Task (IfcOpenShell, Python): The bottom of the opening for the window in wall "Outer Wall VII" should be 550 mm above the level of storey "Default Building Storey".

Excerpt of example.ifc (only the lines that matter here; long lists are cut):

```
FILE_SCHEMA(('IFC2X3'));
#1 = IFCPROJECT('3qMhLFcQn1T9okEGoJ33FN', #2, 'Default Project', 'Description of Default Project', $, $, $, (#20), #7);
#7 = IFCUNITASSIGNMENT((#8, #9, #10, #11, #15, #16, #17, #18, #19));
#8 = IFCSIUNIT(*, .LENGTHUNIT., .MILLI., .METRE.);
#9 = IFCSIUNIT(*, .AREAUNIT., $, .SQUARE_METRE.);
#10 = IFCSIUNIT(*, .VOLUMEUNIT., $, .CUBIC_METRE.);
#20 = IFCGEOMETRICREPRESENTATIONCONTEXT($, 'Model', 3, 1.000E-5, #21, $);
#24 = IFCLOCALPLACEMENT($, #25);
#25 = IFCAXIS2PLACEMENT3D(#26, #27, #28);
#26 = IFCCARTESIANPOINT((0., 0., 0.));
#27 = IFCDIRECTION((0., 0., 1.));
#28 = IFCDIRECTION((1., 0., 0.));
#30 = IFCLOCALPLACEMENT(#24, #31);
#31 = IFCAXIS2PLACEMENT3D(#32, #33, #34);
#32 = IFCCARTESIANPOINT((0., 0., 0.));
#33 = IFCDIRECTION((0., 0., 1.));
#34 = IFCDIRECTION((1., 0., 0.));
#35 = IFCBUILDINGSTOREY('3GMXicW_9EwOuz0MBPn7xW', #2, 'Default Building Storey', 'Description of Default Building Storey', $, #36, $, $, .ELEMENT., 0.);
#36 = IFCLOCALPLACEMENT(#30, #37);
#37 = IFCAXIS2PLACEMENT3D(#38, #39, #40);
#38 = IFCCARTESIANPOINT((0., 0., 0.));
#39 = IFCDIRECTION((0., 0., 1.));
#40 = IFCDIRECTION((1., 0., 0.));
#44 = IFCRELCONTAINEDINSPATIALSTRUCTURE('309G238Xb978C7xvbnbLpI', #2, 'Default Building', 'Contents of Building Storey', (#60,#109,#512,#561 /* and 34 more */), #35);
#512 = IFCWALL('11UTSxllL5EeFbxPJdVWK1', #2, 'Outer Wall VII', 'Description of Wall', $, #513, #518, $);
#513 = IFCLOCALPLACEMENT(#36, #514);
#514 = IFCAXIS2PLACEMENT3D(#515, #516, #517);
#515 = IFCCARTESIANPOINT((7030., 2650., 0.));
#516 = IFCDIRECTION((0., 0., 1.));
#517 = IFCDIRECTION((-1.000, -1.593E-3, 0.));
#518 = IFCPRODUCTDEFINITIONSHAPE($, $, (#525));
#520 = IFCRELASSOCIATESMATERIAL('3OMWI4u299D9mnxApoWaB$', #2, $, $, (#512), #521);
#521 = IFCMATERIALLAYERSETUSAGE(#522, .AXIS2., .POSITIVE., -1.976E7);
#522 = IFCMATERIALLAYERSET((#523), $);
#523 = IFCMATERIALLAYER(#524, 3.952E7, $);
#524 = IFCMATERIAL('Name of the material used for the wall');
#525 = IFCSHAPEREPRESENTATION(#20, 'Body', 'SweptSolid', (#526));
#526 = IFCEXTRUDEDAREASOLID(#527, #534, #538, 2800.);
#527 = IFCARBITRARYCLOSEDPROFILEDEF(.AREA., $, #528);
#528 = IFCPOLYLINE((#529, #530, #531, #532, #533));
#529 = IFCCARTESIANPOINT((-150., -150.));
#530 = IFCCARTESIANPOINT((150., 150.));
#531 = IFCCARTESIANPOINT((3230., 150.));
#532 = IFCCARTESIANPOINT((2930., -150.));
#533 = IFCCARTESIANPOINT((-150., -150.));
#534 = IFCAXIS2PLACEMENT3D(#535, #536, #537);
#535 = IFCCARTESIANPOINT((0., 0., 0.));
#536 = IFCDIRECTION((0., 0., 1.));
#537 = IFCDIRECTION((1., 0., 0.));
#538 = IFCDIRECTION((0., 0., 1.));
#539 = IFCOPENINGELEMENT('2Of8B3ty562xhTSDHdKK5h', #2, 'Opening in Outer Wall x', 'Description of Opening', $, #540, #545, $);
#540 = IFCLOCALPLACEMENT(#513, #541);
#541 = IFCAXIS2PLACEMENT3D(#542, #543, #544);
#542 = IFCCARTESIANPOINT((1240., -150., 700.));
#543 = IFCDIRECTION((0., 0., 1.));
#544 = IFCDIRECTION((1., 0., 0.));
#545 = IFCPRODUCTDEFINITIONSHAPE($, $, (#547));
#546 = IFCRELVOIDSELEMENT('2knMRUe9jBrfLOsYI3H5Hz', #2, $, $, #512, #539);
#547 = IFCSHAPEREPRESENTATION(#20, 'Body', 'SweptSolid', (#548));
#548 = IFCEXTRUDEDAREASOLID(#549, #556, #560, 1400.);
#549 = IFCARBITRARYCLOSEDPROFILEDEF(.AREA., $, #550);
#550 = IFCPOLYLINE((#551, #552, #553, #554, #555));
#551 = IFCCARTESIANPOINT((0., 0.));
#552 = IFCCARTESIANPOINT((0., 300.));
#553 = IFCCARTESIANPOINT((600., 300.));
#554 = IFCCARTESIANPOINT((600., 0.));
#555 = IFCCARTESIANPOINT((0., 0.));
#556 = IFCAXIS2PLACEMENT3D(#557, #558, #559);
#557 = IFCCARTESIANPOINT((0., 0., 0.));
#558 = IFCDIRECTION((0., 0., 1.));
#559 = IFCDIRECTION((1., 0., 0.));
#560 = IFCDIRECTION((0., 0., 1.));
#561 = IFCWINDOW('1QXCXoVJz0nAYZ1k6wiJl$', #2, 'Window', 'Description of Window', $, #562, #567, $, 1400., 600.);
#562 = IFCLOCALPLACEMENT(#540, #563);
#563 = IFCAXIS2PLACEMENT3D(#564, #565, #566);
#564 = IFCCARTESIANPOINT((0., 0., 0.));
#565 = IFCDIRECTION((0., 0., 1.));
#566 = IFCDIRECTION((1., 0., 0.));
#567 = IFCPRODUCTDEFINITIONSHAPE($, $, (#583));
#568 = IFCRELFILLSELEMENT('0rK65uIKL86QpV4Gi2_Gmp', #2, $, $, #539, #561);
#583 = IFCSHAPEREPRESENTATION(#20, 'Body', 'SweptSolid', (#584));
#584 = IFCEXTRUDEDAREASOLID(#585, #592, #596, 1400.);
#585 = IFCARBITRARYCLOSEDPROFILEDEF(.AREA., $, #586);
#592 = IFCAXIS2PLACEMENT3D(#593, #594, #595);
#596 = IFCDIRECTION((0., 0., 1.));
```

```python
import numpy as np
import ifcopenshell
import ifcopenshell.api.geometry
import ifcopenshell.geom
import ifcopenshell.util.element
import ifcopenshell.util.placement
import ifcopenshell.util.shape
import ifcopenshell.util.unit

model = ifcopenshell.open("example.ifc")
unit_scale = ifcopenshell.util.unit.calculate_unit_scale(model)

window = model.by_guid("1QXCXoVJz0nAYZ1k6wiJl$")
opening = window.FillsVoids[0].RelatingOpeningElement
storey = ifcopenshell.util.element.get_container(window, ifc_class="IfcBuildingStorey")
level = ifcopenshell.util.placement.get_local_placement(storey.ObjectPlacement)[2, 3]

# The opening's origin need not be at the sill, so measure its lowest point.
shape = ifcopenshell.geom.create_shape(ifcopenshell.geom.settings(), opening)
bottom = ifcopenshell.util.shape.get_shape_bottom_elevation(shape, shape.geometry) / unit_scale
dz = level + 0.55 / unit_scale - bottom

shift = np.array([0.0, 0.0, dz])
# The window is placed relative to its opening, so it follows when the opening moves.
matrix = ifcopenshell.util.placement.get_local_placement(opening.ObjectPlacement)
matrix[:3, 3] += shift
ifcopenshell.api.geometry.edit_object_placement(
    model, product=opening, matrix=matrix, is_si=False, should_transform_children=True
)

print(f"moved by {dz * unit_scale:+.3f} m")

model.write("example-out.ifc")
```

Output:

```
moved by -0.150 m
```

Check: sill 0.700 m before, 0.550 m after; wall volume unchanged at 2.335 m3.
